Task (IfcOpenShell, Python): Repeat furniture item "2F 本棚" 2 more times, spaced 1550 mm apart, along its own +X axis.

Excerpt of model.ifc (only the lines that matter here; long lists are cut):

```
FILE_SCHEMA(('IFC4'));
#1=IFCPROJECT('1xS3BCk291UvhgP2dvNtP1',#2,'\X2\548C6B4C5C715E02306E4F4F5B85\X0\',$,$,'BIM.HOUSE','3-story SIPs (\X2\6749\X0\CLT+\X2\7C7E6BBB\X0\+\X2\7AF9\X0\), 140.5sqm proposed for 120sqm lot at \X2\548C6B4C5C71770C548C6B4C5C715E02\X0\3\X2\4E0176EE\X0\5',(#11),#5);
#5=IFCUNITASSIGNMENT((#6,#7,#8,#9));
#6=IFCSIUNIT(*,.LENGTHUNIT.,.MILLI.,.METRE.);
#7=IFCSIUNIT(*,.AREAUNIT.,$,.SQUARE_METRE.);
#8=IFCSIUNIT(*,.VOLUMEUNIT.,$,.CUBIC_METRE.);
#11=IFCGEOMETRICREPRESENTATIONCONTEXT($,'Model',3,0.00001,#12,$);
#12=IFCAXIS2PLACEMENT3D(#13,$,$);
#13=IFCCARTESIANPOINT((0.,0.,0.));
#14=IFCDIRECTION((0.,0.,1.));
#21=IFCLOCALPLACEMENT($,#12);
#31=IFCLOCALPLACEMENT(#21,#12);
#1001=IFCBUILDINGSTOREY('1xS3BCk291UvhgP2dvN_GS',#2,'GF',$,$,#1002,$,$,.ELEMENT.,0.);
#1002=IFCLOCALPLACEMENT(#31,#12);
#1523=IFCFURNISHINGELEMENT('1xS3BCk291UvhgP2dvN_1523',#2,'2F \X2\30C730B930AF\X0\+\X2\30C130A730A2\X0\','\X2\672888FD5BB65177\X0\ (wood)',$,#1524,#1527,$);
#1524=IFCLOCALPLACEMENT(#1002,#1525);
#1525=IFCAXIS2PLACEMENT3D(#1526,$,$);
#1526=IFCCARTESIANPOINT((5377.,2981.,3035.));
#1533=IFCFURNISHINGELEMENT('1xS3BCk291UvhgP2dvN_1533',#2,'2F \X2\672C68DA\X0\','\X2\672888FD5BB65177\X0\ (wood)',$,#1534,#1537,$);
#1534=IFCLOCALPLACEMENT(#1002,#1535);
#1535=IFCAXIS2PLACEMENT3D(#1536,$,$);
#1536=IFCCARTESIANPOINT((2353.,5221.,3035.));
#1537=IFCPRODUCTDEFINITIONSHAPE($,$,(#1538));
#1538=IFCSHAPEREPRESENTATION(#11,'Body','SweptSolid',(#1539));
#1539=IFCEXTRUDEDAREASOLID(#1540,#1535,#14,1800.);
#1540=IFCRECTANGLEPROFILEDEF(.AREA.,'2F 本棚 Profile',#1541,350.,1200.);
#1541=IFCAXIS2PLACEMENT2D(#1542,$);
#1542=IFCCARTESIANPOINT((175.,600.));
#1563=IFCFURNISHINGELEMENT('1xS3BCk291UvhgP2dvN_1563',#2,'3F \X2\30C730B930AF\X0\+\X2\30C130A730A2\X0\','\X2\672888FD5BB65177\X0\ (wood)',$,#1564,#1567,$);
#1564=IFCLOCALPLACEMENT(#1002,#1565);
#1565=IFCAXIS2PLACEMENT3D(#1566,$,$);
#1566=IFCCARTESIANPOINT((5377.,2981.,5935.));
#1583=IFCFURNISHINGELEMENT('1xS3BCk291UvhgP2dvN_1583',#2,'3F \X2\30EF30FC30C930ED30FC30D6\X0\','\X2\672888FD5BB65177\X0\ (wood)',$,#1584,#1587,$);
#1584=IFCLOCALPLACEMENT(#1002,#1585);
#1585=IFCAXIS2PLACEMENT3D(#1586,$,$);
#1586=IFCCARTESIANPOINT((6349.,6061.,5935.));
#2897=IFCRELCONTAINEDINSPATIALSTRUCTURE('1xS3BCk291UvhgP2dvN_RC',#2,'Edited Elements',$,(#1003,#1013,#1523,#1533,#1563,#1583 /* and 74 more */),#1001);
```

```python
import ifcopenshell
import ifcopenshell.api.geometry
import ifcopenshell.api.root
import ifcopenshell.util.element
import ifcopenshell.util.placement
import ifcopenshell.util.unit

model = ifcopenshell.open("model.ifc")
unit_scale = ifcopenshell.util.unit.calculate_unit_scale(model)


def reuse_history(source, copy):
    """copy_class also copies each property set's owner history, people and application; keep the originals."""
    for rel in copy.IsDefinedBy:
        if rel.is_a("IfcRelDefinesByProperties") and (history := rel.RelatingPropertyDefinition.OwnerHistory):
            rel.RelatingPropertyDefinition.OwnerHistory = source.OwnerHistory
            ifcopenshell.util.element.remove_deep2(model, history)


source = model.by_guid("1xS3BCk291UvhgP2dvN_1533")
base = ifcopenshell.util.placement.get_local_placement(source.ObjectPlacement)
step = base[:3, 0] * 1.55 / unit_scale

for i in range(1, 3):
    copy = ifcopenshell.api.root.copy_class(model, product=source)
    copy.Representation = ifcopenshell.util.element.copy_deep(
        model, source.Representation, exclude=["IfcGeometricRepresentationContext", "IfcRepresentationMap"]
    )
    reuse_history(source, copy)
    matrix = base.copy()
    matrix[:3, 3] += i * step
    print("added at", matrix[:3, 3].round(3) + 0.0)
    ifcopenshell.api.geometry.edit_object_placement(model, product=copy, matrix=matrix, is_si=False)

model.write("model_v2.ifc")
```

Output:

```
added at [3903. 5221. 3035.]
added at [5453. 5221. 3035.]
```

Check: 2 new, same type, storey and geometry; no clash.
